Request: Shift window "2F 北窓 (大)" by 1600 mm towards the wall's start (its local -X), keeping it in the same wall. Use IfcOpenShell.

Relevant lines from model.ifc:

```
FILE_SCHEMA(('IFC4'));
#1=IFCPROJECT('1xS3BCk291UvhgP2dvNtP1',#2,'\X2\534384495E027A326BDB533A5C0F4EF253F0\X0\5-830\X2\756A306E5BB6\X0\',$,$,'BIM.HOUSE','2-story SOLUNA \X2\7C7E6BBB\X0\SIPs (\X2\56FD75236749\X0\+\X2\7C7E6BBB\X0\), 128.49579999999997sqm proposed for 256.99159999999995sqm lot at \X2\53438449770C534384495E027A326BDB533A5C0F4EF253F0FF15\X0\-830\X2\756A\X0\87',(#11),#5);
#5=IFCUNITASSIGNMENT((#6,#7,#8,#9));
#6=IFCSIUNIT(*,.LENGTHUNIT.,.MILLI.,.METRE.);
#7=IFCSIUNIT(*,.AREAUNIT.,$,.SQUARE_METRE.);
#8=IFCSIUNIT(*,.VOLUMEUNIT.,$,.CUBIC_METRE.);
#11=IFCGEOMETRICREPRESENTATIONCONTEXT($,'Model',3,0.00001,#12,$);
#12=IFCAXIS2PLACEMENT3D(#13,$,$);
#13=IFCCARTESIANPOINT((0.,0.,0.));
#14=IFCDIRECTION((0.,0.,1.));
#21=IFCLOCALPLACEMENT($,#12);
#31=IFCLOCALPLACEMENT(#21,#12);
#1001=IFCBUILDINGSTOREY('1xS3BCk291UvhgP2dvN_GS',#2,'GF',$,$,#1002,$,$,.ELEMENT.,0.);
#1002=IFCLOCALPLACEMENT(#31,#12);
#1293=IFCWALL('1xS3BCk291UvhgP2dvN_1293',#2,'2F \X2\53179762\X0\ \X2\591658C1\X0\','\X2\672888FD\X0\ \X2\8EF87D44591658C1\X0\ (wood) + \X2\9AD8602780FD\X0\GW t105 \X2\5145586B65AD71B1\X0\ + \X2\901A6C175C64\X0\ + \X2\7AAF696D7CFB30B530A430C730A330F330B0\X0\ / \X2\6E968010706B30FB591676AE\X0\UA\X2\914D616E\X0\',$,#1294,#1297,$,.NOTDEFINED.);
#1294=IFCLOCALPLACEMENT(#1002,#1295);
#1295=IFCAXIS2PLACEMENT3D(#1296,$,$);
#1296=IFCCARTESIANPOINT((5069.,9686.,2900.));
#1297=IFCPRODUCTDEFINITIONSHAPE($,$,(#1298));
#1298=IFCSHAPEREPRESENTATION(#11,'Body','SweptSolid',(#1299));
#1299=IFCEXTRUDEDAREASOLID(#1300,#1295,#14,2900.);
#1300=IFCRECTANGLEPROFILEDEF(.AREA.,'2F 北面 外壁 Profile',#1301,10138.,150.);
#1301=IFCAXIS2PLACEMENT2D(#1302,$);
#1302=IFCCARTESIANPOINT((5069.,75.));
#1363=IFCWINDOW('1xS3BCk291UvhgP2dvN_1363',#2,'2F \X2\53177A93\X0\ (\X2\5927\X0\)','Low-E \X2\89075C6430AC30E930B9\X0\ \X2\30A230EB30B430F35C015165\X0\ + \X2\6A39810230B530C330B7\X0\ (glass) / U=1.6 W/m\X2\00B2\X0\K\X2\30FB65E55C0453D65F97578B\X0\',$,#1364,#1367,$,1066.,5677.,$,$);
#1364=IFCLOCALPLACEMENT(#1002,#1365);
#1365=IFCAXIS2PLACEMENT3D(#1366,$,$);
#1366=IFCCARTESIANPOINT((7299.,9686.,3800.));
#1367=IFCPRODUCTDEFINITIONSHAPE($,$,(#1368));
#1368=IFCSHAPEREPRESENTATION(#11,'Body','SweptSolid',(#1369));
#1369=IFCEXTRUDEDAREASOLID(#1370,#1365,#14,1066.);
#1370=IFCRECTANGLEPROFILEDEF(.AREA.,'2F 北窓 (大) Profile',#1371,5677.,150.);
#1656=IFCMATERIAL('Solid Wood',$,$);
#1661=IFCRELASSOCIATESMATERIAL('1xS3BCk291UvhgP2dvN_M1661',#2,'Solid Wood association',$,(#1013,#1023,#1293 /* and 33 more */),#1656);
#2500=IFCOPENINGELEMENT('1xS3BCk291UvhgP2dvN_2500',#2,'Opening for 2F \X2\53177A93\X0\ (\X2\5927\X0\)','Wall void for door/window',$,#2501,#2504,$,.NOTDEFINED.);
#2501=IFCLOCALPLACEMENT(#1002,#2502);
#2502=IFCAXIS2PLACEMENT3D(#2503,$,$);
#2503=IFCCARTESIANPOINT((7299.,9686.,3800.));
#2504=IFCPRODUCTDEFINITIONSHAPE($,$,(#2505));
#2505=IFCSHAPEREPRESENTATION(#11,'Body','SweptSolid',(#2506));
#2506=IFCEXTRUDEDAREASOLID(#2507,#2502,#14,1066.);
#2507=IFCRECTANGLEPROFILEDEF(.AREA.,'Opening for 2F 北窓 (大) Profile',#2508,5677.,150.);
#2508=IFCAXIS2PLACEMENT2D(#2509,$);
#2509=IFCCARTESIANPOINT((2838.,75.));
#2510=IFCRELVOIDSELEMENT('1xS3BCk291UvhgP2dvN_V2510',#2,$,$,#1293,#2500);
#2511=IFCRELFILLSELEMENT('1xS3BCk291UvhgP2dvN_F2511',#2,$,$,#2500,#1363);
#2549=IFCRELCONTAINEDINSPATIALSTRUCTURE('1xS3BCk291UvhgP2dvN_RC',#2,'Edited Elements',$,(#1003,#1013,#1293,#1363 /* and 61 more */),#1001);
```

```python
import ifcopenshell
import ifcopenshell.api.geometry
import ifcopenshell.util.placement

model = ifcopenshell.open("model.ifc")

window = model.by_guid("1xS3BCk291UvhgP2dvN_1363")
opening = window.FillsVoids[0].RelatingOpeningElement
wall = opening.VoidsElements[0].RelatingBuildingElement

wall_matrix = ifcopenshell.util.placement.get_local_placement(wall.ObjectPlacement)
shift = wall_matrix[:3, 0] * -1600.0
before = ifcopenshell.util.placement.get_local_placement(window.ObjectPlacement)[:3, 3].copy()

# The window is not placed relative to its opening, so move both.
for product in (opening, window):
    matrix = ifcopenshell.util.placement.get_local_placement(product.ObjectPlacement)
    matrix[:3, 3] += shift
    ifcopenshell.api.geometry.edit_object_placement(model, product=product, matrix=matrix, is_si=False)

after = ifcopenshell.util.placement.get_local_placement(window.ObjectPlacement)[:3, 3]
print("window moved by", (after - before).round(3) + 0.0)

model.write("model_rev.ifc")
```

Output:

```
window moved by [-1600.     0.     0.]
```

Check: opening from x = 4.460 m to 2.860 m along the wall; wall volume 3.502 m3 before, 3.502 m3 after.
